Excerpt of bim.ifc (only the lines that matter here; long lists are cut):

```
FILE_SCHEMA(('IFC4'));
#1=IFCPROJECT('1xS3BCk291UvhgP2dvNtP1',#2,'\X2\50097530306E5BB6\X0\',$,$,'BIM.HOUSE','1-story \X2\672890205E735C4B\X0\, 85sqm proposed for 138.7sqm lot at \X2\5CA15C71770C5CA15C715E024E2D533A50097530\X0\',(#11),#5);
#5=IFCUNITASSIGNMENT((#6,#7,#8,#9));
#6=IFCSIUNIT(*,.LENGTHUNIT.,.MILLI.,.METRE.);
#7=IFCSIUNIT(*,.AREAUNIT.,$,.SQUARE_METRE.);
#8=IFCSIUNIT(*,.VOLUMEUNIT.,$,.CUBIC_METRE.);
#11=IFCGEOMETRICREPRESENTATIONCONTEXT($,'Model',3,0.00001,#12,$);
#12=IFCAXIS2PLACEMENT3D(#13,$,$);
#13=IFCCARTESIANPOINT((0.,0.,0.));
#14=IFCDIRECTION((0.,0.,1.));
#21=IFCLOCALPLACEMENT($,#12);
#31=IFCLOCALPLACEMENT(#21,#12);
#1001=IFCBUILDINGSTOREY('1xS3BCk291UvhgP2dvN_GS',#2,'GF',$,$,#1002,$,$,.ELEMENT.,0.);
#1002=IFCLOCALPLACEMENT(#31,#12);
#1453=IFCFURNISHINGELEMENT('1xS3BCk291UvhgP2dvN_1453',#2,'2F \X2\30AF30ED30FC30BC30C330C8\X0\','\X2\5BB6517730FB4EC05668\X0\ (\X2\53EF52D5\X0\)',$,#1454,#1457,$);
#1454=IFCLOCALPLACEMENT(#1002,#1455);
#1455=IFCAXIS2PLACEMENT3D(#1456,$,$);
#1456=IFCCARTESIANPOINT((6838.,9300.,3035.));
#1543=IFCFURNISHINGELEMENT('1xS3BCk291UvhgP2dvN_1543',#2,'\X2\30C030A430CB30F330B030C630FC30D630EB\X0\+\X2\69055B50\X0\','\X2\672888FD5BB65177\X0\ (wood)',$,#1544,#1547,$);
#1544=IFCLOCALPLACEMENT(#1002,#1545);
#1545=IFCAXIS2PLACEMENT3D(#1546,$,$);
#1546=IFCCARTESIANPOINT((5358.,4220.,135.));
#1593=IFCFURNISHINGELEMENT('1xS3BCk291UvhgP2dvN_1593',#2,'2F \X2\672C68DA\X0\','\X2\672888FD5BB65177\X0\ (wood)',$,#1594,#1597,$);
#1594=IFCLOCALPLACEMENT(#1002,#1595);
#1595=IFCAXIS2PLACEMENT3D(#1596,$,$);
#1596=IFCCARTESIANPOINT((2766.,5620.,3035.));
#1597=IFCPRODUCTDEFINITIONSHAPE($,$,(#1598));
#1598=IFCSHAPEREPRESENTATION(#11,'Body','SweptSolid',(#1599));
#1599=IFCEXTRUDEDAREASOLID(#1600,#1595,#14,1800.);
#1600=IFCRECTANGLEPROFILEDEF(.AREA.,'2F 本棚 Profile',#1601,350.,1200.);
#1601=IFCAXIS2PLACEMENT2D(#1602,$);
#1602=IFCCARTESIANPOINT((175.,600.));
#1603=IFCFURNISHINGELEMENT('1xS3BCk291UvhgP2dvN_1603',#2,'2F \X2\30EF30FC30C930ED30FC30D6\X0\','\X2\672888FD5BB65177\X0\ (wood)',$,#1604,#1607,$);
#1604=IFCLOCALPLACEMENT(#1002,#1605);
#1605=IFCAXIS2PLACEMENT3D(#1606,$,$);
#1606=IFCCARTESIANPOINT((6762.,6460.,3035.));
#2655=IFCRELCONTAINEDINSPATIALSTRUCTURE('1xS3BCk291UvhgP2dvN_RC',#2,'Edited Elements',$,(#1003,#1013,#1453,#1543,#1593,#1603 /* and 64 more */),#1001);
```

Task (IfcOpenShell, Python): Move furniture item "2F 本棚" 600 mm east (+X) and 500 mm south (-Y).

```python
import ifcopenshell
import ifcopenshell.api.geometry
import ifcopenshell.util.placement
import ifcopenshell.util.unit

model = ifcopenshell.open("bim.ifc")
unit_scale = ifcopenshell.util.unit.calculate_unit_scale(model)

item = model.by_id(1593)
matrix = ifcopenshell.util.placement.get_local_placement(item.ObjectPlacement)
matrix[0, 3] += 0.6 / unit_scale
matrix[1, 3] -= 0.5 / unit_scale
ifcopenshell.api.geometry.edit_object_placement(model, product=item, matrix=matrix, is_si=False)

print(ifcopenshell.util.placement.get_local_placement(item.ObjectPlacement).round(3) + 0.0)

model.write("bim_rev.ifc")
```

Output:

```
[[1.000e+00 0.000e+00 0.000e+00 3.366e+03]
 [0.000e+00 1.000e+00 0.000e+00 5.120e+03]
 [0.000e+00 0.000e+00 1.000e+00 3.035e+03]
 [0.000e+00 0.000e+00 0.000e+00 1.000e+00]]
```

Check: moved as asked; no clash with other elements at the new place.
